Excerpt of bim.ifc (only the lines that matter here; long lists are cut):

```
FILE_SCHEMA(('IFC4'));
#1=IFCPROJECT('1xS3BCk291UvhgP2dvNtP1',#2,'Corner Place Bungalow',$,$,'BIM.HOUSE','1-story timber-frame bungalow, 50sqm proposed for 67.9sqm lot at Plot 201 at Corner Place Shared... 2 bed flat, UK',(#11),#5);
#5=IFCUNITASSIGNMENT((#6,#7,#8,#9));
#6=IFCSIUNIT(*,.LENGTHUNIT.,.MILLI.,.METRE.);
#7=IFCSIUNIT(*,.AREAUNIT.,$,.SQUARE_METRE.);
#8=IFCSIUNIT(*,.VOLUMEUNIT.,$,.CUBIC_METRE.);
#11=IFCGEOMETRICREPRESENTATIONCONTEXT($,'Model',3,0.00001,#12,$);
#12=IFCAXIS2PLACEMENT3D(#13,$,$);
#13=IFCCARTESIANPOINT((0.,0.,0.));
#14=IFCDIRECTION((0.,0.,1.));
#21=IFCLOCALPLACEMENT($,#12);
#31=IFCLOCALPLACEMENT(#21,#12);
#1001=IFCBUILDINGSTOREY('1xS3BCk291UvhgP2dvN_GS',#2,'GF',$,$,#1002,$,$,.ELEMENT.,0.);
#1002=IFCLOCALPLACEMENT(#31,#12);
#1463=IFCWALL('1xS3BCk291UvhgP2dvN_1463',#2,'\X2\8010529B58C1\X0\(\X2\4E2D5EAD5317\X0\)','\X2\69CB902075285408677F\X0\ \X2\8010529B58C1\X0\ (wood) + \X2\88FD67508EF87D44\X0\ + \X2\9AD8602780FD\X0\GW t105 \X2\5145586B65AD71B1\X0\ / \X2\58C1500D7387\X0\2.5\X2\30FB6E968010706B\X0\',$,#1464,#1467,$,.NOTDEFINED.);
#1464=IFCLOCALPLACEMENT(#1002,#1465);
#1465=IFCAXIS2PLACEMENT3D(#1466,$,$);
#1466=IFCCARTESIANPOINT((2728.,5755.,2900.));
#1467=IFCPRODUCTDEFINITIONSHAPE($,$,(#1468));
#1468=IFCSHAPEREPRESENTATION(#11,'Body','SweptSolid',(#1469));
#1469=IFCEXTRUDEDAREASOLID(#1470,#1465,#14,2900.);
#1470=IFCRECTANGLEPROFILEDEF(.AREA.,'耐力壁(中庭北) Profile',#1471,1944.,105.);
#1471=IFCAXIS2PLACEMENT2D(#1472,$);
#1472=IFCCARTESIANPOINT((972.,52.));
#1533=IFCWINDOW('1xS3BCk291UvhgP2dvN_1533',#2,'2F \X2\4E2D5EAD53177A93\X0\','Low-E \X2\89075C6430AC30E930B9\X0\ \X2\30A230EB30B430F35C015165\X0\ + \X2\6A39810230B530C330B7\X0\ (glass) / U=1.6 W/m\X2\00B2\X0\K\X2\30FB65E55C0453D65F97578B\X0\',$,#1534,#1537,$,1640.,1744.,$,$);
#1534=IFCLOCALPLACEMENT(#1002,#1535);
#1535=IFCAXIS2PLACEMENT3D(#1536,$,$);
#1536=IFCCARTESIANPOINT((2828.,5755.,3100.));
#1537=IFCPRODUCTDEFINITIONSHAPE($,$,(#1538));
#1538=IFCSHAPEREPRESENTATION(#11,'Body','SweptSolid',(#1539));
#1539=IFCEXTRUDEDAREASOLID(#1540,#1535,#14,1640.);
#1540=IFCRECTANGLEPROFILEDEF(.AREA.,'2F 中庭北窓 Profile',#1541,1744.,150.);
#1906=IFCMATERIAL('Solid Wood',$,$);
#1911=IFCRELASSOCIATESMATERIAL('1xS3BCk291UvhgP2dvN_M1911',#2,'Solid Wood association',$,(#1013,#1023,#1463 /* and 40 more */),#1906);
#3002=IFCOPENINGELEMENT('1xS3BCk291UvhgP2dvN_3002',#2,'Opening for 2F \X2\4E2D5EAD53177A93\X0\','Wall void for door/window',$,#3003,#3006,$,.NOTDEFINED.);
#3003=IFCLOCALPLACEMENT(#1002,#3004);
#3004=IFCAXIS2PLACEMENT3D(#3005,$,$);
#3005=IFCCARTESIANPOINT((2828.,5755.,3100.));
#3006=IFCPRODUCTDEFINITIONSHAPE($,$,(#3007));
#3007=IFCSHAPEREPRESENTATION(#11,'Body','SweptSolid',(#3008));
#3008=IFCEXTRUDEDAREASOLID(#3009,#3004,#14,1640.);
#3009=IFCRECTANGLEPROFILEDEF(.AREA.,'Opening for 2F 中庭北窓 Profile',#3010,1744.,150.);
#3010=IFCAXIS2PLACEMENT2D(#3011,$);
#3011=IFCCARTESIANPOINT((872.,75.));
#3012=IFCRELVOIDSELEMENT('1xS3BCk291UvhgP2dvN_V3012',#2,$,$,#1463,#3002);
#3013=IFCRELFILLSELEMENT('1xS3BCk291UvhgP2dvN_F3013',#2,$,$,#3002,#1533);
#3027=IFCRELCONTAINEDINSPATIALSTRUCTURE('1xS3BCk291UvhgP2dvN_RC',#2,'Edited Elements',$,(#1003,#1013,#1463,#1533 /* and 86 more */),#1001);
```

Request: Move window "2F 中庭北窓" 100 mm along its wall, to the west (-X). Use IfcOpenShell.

```python
import ifcopenshell
import ifcopenshell.api.geometry
import ifcopenshell.util.placement

model = ifcopenshell.open("bim.ifc")

window = model.by_guid("1xS3BCk291UvhgP2dvN_1533")
opening = window.FillsVoids[0].RelatingOpeningElement
wall = opening.VoidsElements[0].RelatingBuildingElement

wall_matrix = ifcopenshell.util.placement.get_local_placement(wall.ObjectPlacement)
shift = wall_matrix[:3, 0] * -100.0
before = ifcopenshell.util.placement.get_local_placement(window.ObjectPlacement)[:3, 3].copy()

# The window is not placed relative to its opening, so move both.
for product in (opening, window):
    matrix = ifcopenshell.util.placement.get_local_placement(product.ObjectPlacement)
    matrix[:3, 3] += shift
    ifcopenshell.api.geometry.edit_object_placement(model, product=product, matrix=matrix, is_si=False)

after = ifcopenshell.util.placement.get_local_placement(window.ObjectPlacement)[:3, 3]
print("window moved by", (after - before).round(3) + 0.0)

model.write("bim_rev.ifc")
```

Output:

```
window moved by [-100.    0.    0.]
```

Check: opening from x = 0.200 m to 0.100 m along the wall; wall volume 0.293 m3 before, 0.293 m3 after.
